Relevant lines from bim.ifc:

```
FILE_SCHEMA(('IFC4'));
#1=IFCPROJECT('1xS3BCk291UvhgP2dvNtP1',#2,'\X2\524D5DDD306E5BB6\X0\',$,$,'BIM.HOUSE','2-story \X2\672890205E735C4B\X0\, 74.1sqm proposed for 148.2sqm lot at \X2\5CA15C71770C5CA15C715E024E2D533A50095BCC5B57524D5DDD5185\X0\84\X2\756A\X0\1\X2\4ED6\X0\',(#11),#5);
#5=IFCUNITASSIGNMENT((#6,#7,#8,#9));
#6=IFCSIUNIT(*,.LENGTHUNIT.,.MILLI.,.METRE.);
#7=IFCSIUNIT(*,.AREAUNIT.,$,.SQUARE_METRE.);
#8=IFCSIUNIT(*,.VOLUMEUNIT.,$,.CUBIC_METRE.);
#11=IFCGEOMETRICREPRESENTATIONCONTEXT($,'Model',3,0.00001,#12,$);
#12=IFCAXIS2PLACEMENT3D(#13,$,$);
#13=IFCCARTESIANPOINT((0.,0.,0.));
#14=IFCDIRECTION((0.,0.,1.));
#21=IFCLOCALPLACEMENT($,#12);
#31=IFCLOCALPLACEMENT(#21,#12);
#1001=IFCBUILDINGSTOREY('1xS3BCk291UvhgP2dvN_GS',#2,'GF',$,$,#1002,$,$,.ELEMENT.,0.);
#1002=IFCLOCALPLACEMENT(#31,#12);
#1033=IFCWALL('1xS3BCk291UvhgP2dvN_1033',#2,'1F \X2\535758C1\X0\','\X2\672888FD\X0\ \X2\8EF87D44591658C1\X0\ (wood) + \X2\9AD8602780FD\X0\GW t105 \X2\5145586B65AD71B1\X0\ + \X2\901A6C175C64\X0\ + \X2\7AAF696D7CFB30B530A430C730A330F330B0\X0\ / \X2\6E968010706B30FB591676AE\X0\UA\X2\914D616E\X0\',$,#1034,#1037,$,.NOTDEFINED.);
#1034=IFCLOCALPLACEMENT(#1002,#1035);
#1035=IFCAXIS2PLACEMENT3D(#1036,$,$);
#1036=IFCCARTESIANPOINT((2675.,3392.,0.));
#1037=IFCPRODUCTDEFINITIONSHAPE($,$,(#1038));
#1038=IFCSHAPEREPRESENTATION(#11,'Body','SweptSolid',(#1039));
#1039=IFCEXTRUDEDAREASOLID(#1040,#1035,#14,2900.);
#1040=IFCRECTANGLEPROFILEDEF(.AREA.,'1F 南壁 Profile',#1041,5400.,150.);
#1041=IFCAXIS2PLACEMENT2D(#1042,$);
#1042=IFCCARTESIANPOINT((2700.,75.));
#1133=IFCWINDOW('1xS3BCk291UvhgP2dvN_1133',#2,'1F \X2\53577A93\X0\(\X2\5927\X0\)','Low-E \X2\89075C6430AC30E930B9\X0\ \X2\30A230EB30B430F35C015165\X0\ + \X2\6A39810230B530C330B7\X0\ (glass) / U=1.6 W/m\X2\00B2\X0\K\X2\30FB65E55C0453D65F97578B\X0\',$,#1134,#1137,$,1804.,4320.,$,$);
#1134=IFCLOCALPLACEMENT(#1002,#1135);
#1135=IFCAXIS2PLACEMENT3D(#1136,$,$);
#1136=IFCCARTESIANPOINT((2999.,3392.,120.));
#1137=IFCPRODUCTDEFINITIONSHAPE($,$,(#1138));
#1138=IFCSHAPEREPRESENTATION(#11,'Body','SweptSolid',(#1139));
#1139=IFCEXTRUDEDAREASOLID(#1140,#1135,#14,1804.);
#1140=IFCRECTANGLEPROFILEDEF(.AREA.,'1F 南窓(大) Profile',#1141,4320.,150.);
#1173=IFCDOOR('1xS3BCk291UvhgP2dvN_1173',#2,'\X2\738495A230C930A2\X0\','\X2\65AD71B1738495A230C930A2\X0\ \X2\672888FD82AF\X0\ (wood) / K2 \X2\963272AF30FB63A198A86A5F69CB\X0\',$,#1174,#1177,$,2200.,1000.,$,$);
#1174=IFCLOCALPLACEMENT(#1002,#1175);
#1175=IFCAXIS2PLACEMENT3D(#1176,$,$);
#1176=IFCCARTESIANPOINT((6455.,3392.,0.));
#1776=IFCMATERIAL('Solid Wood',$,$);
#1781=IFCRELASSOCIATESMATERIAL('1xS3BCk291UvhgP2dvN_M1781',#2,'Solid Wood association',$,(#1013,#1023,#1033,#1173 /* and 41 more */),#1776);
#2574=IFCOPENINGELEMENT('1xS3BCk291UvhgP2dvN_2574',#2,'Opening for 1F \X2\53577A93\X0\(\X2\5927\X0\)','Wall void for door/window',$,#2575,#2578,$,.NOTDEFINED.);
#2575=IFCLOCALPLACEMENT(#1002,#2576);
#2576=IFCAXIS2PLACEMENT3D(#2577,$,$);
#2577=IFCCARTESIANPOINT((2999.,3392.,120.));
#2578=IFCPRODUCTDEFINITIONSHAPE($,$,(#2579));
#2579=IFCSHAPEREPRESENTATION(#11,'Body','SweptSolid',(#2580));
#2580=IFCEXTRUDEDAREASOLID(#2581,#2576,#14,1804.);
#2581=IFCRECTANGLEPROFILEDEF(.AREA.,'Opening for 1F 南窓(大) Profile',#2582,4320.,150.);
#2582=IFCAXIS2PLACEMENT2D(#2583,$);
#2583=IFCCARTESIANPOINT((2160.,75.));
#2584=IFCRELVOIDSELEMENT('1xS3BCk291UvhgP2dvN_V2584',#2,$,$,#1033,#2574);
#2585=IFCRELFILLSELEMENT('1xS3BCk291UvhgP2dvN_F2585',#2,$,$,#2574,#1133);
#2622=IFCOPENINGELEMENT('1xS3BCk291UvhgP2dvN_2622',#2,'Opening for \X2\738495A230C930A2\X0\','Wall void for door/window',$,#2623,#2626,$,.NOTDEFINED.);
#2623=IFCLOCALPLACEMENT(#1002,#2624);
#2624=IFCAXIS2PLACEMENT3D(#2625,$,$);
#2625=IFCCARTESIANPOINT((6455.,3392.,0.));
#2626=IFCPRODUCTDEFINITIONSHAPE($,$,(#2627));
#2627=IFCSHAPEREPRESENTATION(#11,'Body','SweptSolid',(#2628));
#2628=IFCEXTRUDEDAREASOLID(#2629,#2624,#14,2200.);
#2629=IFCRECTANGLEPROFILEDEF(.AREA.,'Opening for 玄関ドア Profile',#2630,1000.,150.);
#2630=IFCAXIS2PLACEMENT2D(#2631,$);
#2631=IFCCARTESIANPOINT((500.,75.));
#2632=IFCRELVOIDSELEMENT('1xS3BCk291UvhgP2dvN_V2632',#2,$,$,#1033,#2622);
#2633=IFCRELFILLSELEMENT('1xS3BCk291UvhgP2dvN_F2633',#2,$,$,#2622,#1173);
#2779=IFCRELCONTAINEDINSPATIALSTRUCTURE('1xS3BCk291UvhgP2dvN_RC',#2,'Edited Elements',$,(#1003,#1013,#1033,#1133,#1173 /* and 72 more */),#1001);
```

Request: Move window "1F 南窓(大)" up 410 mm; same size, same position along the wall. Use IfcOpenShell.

```python
import numpy as np
import ifcopenshell
import ifcopenshell.api.geometry
import ifcopenshell.util.placement
import ifcopenshell.util.unit

model = ifcopenshell.open("bim.ifc")
unit_scale = ifcopenshell.util.unit.calculate_unit_scale(model)

window = model.by_guid("1xS3BCk291UvhgP2dvN_1133")
opening = window.FillsVoids[0].RelatingOpeningElement
dz = 0.41 / unit_scale

shift = np.array([0.0, 0.0, dz])
# The window is not placed relative to its opening, so move both.
for product in (opening, window):
    matrix = ifcopenshell.util.placement.get_local_placement(product.ObjectPlacement)
    matrix[:3, 3] += shift
    ifcopenshell.api.geometry.edit_object_placement(model, product=product, matrix=matrix, is_si=False)

print(f"moved by {dz * unit_scale:+.3f} m")

model.write("bim_edited.ifc")
```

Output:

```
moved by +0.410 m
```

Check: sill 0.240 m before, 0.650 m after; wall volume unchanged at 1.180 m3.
